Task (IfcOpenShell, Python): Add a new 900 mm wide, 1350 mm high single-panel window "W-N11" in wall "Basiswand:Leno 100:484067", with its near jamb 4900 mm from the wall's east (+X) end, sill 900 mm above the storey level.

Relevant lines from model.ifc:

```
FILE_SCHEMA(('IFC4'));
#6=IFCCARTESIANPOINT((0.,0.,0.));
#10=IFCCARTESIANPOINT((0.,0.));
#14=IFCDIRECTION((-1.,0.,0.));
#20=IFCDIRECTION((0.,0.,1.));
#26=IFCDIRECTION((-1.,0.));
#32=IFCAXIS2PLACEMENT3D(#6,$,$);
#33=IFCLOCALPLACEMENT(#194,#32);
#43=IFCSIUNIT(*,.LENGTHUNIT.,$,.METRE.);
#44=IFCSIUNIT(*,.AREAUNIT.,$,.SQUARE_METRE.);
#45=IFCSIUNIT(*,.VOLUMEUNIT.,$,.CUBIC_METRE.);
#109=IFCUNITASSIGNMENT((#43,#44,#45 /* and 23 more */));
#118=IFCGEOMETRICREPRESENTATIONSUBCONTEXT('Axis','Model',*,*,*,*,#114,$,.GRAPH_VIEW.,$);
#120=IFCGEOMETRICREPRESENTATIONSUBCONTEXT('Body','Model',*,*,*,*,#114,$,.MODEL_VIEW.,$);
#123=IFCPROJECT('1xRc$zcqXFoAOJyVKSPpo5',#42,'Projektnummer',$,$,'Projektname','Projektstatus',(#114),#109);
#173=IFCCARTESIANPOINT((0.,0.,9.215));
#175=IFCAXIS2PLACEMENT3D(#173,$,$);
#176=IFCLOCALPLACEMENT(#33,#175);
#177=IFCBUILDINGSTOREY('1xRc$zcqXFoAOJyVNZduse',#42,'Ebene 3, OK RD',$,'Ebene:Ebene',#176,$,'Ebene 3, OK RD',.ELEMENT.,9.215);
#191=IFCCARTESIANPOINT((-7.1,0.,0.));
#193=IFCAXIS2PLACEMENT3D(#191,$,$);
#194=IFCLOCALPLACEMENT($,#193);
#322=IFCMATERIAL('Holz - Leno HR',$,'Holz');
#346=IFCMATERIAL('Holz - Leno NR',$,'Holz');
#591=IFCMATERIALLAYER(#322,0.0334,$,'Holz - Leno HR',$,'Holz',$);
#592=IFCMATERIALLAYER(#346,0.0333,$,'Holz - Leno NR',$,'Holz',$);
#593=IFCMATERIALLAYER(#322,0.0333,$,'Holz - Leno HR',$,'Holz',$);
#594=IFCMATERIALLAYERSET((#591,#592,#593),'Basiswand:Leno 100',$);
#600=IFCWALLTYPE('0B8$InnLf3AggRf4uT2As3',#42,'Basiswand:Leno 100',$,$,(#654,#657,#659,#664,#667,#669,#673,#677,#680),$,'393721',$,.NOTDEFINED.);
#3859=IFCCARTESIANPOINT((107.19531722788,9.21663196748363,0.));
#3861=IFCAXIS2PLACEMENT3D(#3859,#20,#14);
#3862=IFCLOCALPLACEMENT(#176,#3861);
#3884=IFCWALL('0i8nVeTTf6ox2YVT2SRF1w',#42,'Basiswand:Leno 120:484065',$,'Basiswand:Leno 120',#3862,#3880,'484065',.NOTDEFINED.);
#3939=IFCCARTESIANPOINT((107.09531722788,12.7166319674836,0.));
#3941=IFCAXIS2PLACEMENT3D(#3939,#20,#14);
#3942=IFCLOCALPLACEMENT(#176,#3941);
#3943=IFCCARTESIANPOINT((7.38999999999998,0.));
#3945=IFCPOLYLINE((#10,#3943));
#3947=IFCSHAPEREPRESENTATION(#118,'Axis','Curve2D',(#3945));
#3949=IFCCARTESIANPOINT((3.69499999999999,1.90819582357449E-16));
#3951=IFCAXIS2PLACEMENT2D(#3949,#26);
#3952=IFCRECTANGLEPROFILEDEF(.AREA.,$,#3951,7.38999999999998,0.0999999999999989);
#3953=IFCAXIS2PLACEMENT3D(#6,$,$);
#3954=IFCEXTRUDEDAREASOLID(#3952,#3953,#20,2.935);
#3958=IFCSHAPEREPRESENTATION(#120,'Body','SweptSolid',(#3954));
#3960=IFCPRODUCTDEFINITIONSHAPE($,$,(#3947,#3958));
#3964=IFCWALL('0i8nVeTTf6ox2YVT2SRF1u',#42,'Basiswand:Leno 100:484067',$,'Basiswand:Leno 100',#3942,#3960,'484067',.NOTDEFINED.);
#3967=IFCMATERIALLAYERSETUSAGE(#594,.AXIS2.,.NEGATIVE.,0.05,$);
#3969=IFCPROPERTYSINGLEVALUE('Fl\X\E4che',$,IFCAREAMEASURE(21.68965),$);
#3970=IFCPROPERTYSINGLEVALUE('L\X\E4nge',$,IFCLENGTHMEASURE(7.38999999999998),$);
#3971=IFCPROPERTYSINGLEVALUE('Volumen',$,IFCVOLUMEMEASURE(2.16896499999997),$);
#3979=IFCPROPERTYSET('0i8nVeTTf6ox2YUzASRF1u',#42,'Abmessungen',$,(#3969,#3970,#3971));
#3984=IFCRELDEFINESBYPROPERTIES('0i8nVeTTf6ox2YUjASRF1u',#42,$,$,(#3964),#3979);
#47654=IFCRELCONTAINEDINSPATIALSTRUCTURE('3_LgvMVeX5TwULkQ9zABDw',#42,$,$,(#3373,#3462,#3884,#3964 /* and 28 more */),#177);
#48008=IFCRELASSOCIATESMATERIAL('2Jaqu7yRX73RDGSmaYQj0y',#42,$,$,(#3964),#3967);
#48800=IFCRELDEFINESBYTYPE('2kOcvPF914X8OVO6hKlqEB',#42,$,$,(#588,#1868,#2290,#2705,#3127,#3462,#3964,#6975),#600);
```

```python
import numpy as np
import ifcopenshell
import ifcopenshell.api.feature
import ifcopenshell.api.geometry
import ifcopenshell.api.pset
import ifcopenshell.api.root
import ifcopenshell.api.spatial
import ifcopenshell.geom
import ifcopenshell.util.element
import ifcopenshell.util.placement
import ifcopenshell.util.representation
import ifcopenshell.util.shape
import ifcopenshell.util.unit

model = ifcopenshell.open("model.ifc")
unit_scale = ifcopenshell.util.unit.calculate_unit_scale(model)
area_scale = ifcopenshell.util.unit.calculate_unit_scale(model, "AREAUNIT")
volume_scale = ifcopenshell.util.unit.calculate_unit_scale(model, "VOLUMEUNIT")
settings = ifcopenshell.geom.settings()


def volume(element):
    """Net volume in cubic metres, openings subtracted."""
    shape = ifcopenshell.geom.create_shape(settings, element)
    return ifcopenshell.util.shape.get_volume(shape.geometry)


wall = model.by_guid("0i8nVeTTf6ox2YVT2SRF1u")
storey = ifcopenshell.util.element.get_container(wall, ifc_class="IfcBuildingStorey")
context = ifcopenshell.util.representation.get_context(model, "Model", "Body", "MODEL_VIEW")
before = volume(wall)

width, height, from_end, sill = 0.9, 1.35, 4.9, 0.9  # metres

# The wall runs along its own X axis, and the end named is its -X end.
wall_shape = ifcopenshell.geom.create_shape(settings, wall)
x, y, z = ifcopenshell.util.shape.get_vertices(wall_shape.geometry).T
start = x.min() + from_end
face, thickness = float(y.min()), float(y.max() - y.min())
wall_matrix = ifcopenshell.util.placement.get_local_placement(wall.ObjectPlacement)
level = ifcopenshell.util.placement.get_local_placement(storey.ObjectPlacement)[2, 3]


def in_wall(x, y):
    """Placement at x, y metres in the wall's axes, at sill height."""
    matrix = wall_matrix.copy()
    matrix[:, 3] = wall_matrix @ np.array([x / unit_scale, y / unit_scale, 0.0, 1.0])
    matrix[2, 3] = level + sill / unit_scale
    return matrix


# Opening: a box that overshoots both wall faces by 50 mm.
opening = ifcopenshell.api.root.create_entity(model, ifc_class="IfcOpeningElement", predefined_type="OPENING")
box = ifcopenshell.api.geometry.add_wall_representation(
    model, context=context, length=width, height=height, thickness=thickness + 0.1
)
ifcopenshell.api.geometry.assign_representation(model, product=opening, representation=box)
ifcopenshell.api.geometry.edit_object_placement(model, product=opening, matrix=in_wall(start, face - 0.05), is_si=False)
ifcopenshell.api.feature.add_feature(model, feature=opening, element=wall)

window = ifcopenshell.api.root.create_entity(model, ifc_class="IfcWindow", name="W-N11", predefined_type="WINDOW")
window.OverallWidth, window.OverallHeight = width / unit_scale, height / unit_scale
window.PartitioningType = "SINGLE_PANEL"
body = ifcopenshell.api.geometry.add_window_representation(
    model,
    context=context,
    overall_width=window.OverallWidth,
    overall_height=window.OverallHeight,
    partition_type="SINGLE_PANEL",
)
ifcopenshell.api.geometry.assign_representation(model, product=window, representation=body)
ifcopenshell.api.spatial.assign_container(model, products=[window], relating_structure=storey)
ifcopenshell.api.feature.add_filling(model, opening=opening, element=window)

# Centre the window in the wall's thickness.
ifcopenshell.api.geometry.edit_object_placement(model, product=window, matrix=in_wall(start, face), is_si=False)
window_shape = ifcopenshell.geom.create_shape(settings, window)
depth = ifcopenshell.util.shape.get_vertices(window_shape.geometry)[:, 1]
offset = face + thickness / 2 - (depth.min() + depth.max()) / 2
ifcopenshell.api.geometry.edit_object_placement(model, product=window, matrix=in_wall(start, offset), is_si=False)

after = volume(wall)

# Update the wall's stored quantities.
pset = model.by_id(ifcopenshell.util.element.get_pset(wall, "Abmessungen", should_inherit=False)["id"])
ifcopenshell.api.pset.edit_pset(model, pset=pset, properties={
    "Fläche": model.create_entity("IfcAreaMeasure", after / thickness / area_scale),
    "Volumen": model.create_entity("IfcVolumeMeasure", after / volume_scale),
})

print(f"wall volume {before:.3f} -> {after:.3f} m3")

model.write("model_rev.ifc")
```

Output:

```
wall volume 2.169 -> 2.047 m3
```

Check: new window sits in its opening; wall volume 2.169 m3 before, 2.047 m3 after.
